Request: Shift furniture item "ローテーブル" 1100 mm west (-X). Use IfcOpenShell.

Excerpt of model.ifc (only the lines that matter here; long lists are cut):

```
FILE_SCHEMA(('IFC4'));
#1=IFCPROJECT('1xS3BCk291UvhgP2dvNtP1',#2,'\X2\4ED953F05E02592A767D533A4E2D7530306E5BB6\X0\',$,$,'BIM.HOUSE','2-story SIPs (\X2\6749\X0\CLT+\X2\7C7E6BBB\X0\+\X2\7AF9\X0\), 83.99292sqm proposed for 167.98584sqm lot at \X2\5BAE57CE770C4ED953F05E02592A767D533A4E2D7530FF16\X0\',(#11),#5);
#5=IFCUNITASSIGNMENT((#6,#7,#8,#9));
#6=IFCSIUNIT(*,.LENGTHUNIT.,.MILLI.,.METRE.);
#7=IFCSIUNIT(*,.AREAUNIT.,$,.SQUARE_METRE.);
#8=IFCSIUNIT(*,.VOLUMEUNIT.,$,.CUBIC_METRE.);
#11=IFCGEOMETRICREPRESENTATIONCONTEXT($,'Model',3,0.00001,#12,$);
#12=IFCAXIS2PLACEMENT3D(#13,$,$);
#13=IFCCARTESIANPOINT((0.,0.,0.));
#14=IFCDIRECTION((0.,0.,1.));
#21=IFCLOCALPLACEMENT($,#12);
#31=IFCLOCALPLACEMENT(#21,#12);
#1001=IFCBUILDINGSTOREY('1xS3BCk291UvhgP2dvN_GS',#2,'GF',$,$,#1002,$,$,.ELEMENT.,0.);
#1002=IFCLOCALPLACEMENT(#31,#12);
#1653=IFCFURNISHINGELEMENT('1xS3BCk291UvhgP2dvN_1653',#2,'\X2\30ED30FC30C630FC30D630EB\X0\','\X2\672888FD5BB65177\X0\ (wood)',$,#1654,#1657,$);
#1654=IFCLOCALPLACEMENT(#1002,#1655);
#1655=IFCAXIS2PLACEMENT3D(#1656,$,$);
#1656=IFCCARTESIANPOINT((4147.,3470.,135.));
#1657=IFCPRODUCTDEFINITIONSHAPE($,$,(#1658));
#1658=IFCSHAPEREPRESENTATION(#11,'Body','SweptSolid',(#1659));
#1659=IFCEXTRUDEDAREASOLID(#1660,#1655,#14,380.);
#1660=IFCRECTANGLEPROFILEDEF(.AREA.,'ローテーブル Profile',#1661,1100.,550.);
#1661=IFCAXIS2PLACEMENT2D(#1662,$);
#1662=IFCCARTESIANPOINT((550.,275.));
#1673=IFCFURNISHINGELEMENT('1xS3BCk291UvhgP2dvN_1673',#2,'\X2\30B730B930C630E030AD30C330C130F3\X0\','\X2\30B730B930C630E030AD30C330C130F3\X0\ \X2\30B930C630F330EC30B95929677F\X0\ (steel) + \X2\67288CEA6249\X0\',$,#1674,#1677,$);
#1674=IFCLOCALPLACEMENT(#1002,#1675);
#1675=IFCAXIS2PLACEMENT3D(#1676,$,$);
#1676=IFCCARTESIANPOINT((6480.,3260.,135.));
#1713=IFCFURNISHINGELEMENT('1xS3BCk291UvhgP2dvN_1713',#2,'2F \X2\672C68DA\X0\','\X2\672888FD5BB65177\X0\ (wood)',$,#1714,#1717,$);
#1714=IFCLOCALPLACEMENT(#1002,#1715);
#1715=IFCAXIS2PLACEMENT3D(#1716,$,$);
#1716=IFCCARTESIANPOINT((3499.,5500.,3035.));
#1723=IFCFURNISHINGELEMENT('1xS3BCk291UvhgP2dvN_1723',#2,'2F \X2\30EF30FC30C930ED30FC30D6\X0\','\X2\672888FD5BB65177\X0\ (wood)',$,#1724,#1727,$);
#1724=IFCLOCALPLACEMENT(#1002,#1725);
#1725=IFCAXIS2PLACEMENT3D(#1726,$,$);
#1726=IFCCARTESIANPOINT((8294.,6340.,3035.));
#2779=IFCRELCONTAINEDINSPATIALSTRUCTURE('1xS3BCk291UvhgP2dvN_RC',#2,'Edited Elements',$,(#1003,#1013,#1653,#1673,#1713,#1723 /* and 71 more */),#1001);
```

```python
import ifcopenshell
import ifcopenshell.api.geometry
import ifcopenshell.util.placement

model = ifcopenshell.open("model.ifc")

item = model.by_guid("1xS3BCk291UvhgP2dvN_1653")
matrix = ifcopenshell.util.placement.get_local_placement(item.ObjectPlacement)
matrix[0, 3] -= 1100.0
ifcopenshell.api.geometry.edit_object_placement(model, product=item, matrix=matrix, is_si=False)

print(ifcopenshell.util.placement.get_local_placement(item.ObjectPlacement).round(3) + 0.0)

model.write("model_rev.ifc")
```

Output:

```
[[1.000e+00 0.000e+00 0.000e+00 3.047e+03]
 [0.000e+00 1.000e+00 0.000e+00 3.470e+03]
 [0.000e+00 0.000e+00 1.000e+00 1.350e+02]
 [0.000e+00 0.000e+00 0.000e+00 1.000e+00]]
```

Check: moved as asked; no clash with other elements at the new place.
